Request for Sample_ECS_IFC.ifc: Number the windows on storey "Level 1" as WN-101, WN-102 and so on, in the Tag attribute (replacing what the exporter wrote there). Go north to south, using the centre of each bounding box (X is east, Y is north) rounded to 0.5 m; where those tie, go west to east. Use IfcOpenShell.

First a look at what the model holds.

```python
import ifcopenshell
import ifcopenshell.util.element
import ifcopenshell.util.placement

model = ifcopenshell.open("Sample_ECS_IFC.ifc")
print(model.schema)
storey = next(s for s in model.by_type("IfcBuildingStorey") if s.Name == "Level 1")
windows = [e for e in ifcopenshell.util.element.get_decomposition(storey) if e.is_a("IfcWindow")]
for e in sorted(windows, key=lambda e: e.id()):
    origin = ifcopenshell.util.placement.get_local_placement(e.ObjectPlacement)[:3, 3]
    print(e.id(), e.Tag, e.Name, origin.round(2) + 0.0, sep=" | ")
```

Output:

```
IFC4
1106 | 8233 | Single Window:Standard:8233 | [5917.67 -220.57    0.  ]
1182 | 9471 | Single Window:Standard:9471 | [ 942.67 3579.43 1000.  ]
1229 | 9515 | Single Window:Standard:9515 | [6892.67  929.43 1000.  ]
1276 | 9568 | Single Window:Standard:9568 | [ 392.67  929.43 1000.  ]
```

```python
import ifcopenshell
import ifcopenshell.geom
import ifcopenshell.util.element
import ifcopenshell.util.shape

model = ifcopenshell.open("Sample_ECS_IFC.ifc")
settings = ifcopenshell.geom.settings()
settings.set("use-world-coords", True)


def centre(element):
    shape = ifcopenshell.geom.create_shape(settings, element)
    return ifcopenshell.util.shape.get_bbox_centroid(shape.geometry)


storey = next(s for s in model.by_type("IfcBuildingStorey") if s.Name == "Level 1")
windows = [e for e in ifcopenshell.util.element.get_decomposition(storey) if e.is_a("IfcWindow")]

# Insertion points can sit at a corner or the storey origin, so sort by the geometry (in metres).
centres = {e: centre(e) for e in windows}
windows.sort(key=lambda e: (-round(centres[e][1] / 0.5), centres[e][0]))

for i, e in enumerate(windows, start=1):
    number = f"WN-1{i:02d}"
    e.Tag = number
    print(e.id(), number)

model.write("Sample_ECS_IFC_edited.ifc")
```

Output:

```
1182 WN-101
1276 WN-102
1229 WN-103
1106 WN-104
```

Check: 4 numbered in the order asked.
